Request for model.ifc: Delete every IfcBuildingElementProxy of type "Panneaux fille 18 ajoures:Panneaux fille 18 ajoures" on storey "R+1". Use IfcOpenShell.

First a look at what the model holds.

```python
import ifcopenshell
import ifcopenshell.util.element

model = ifcopenshell.open("model.ifc")
print(model.schema)
storey = next(s for s in model.by_type("IfcBuildingStorey") if s.Name == "R+1")
proxies = [e for e in ifcopenshell.util.element.get_decomposition(storey) if e.is_a("IfcBuildingElementProxy")]
seen = {}
for e in proxies:
    element_type = ifcopenshell.util.element.get_type(e)
    name = element_type.Name if element_type not in (None, e) else None
    seen[name] = seen.get(name, 0) + 1
for name, count in sorted(seen.items(), key=str):
    print(count, "x", name)
```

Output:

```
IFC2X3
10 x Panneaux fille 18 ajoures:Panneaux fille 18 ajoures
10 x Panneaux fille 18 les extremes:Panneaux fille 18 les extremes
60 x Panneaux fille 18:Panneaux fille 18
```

```python
import ifcopenshell
import ifcopenshell.api.root
import ifcopenshell.util.element

model = ifcopenshell.open("model.ifc")

storey = next(s for s in model.by_type("IfcBuildingStorey") if s.Name == "R+1")
proxies = [e for e in ifcopenshell.util.element.get_decomposition(storey) if e.is_a("IfcBuildingElementProxy")]
targets = [e for e in proxies if (t := ifcopenshell.util.element.get_type(e)) not in (None, e) and t.Name == "Panneaux fille 18 ajoures:Panneaux fille 18 ajoures"]

for e in targets:
    ifcopenshell.api.root.remove_product(model, product=e)
print(len(targets), "removed")

model.write("model_edited.ifc")
```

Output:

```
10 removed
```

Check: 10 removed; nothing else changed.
